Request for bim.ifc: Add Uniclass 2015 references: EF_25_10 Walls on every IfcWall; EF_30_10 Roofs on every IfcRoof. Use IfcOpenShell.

First a look at what the model holds.

```python
import ifcopenshell

model = ifcopenshell.open("bim.ifc")
print(model.schema)
print("classifications:", [c.Name for c in model.by_type("IfcClassification")])
for ifc_class in ("IfcDoor", "IfcRoof", "IfcStair", "IfcWall", "IfcWindow"):
    print(ifc_class, len(model.by_type(ifc_class)))
```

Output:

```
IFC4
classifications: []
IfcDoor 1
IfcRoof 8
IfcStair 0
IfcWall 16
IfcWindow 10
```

```python
import ifcopenshell
import ifcopenshell.api.classification

model = ifcopenshell.open("bim.ifc")

system = ifcopenshell.api.classification.add_classification(model, classification="Uniclass 2015")

codes = {
    "IfcWall": ("EF_25_10", "Walls"),
    "IfcRoof": ("EF_30_10", "Roofs"),
}
for ifc_class, (code, name) in codes.items():
    products = model.by_type(ifc_class)
    ifcopenshell.api.classification.add_reference(
        model, products=products, classification=system, identification=code, name=name
    )
    print(code, len(products))

model.write("bim_edited.ifc")
```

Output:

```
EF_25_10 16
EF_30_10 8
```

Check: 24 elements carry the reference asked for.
